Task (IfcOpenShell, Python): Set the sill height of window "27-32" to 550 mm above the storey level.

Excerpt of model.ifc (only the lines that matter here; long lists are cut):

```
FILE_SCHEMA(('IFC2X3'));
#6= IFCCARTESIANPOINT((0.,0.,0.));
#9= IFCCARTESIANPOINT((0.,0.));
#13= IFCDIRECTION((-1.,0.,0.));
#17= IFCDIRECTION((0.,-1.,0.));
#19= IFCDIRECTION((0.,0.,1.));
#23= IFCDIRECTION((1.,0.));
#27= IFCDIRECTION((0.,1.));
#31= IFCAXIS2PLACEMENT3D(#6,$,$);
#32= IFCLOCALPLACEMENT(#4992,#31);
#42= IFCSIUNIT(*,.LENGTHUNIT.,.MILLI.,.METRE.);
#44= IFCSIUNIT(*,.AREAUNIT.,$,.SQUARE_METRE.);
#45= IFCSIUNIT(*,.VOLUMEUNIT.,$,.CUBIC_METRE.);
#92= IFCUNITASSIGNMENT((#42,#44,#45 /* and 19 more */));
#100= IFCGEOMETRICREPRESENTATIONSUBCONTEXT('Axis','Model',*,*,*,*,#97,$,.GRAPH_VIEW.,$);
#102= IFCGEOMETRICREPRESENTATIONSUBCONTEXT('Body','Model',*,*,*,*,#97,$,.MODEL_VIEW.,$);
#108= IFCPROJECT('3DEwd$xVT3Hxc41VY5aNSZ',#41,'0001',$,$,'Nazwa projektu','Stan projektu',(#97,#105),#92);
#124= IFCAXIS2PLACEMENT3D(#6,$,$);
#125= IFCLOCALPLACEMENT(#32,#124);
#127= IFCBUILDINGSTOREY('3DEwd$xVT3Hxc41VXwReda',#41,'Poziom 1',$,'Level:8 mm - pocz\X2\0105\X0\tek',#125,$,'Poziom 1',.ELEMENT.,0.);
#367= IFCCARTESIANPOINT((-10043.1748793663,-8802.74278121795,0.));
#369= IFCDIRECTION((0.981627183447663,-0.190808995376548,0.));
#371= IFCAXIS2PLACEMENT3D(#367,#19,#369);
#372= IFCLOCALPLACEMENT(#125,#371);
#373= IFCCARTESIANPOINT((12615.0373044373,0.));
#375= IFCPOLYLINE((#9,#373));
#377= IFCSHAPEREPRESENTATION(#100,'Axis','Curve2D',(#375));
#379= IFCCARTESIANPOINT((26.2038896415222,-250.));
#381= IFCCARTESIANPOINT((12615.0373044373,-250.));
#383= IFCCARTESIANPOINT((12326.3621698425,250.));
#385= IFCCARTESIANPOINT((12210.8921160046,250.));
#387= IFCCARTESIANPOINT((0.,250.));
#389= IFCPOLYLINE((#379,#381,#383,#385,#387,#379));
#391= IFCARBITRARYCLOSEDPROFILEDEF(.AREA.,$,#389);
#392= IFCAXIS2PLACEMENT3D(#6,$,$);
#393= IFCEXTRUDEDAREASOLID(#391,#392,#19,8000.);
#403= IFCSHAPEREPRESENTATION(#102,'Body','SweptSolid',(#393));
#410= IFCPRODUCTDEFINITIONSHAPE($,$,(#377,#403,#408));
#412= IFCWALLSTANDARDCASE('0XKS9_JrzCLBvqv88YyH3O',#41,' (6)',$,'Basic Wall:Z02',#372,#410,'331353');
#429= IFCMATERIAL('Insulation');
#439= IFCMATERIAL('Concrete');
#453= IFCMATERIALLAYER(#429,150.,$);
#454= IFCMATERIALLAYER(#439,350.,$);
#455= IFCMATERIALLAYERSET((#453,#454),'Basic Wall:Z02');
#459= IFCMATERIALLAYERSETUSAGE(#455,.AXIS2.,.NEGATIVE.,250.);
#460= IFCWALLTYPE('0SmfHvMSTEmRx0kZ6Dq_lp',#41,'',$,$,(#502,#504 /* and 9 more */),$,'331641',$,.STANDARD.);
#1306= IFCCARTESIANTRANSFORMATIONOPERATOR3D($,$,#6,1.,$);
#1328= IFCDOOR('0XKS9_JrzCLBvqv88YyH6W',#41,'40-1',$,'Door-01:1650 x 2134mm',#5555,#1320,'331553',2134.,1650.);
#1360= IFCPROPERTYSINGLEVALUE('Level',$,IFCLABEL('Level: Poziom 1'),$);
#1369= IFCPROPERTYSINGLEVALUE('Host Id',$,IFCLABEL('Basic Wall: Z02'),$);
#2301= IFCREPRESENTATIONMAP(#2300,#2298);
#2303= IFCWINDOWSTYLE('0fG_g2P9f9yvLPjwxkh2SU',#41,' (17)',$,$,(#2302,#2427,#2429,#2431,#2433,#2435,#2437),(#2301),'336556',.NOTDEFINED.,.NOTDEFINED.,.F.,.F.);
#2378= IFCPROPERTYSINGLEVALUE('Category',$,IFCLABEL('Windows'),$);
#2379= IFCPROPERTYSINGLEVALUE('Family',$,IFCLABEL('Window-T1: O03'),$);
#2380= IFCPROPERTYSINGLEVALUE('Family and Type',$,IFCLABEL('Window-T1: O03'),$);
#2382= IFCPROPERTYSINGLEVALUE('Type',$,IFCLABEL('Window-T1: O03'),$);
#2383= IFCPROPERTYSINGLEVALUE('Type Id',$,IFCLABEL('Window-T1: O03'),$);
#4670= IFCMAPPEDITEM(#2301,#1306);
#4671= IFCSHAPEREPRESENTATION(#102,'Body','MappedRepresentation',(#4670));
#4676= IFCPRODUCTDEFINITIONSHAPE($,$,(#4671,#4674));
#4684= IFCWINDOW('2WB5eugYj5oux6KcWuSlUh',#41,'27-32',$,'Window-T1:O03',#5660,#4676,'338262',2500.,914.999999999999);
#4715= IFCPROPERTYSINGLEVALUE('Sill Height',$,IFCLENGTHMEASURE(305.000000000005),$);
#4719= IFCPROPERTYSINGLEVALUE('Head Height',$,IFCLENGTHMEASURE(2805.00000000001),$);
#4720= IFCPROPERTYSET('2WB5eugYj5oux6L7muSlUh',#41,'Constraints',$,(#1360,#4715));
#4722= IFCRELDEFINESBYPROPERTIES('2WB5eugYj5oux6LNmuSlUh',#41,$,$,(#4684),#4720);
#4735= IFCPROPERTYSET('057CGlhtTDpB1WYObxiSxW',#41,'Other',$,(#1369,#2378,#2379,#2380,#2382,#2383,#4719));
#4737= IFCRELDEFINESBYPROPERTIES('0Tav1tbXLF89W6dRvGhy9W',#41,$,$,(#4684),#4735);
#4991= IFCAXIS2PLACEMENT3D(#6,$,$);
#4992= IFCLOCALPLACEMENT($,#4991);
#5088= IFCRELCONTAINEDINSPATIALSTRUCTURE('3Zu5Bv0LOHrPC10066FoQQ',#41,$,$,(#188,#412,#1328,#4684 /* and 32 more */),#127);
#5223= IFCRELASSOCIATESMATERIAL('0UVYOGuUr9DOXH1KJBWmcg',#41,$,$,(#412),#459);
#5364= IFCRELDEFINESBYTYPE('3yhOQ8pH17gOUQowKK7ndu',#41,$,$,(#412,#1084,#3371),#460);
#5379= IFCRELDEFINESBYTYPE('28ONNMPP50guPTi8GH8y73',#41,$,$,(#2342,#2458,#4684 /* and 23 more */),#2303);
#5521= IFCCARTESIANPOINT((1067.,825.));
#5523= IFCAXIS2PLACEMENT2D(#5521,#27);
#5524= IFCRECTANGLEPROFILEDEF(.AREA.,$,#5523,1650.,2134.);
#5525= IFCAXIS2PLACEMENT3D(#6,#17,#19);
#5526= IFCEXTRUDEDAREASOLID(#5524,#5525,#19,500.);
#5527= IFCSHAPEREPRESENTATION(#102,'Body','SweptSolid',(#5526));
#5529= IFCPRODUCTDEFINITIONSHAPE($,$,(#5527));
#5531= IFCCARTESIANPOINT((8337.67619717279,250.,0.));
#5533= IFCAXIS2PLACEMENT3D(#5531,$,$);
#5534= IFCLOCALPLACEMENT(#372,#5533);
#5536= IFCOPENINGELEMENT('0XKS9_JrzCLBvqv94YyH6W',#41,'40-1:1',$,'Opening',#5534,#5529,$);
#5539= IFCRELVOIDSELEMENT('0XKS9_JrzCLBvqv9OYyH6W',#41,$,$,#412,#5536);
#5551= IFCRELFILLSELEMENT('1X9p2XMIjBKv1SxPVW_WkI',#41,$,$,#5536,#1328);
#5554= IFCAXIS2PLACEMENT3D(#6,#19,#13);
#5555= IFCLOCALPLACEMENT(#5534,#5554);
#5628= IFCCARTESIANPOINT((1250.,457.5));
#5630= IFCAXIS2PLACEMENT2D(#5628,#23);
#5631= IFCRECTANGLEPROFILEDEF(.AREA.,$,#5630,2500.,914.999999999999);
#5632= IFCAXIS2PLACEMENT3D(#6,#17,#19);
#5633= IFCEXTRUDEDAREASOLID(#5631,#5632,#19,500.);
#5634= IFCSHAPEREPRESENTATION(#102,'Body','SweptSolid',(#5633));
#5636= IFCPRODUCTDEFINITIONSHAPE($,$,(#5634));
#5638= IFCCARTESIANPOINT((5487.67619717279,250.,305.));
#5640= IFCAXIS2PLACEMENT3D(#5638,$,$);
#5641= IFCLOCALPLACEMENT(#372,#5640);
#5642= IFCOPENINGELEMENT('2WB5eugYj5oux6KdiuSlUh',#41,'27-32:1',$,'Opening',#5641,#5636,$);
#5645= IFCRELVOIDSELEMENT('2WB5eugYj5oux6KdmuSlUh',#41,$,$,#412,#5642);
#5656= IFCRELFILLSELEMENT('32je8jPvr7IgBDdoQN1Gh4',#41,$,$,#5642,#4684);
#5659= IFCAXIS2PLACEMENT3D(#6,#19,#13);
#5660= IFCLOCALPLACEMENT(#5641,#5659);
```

```python
import numpy as np
import ifcopenshell
import ifcopenshell.api.geometry
import ifcopenshell.api.pset
import ifcopenshell.geom
import ifcopenshell.util.element
import ifcopenshell.util.placement
import ifcopenshell.util.shape
import ifcopenshell.util.unit

model = ifcopenshell.open("model.ifc")
unit_scale = ifcopenshell.util.unit.calculate_unit_scale(model)

window = model.by_guid("2WB5eugYj5oux6KcWuSlUh")
opening = window.FillsVoids[0].RelatingOpeningElement
storey = ifcopenshell.util.element.get_container(window, ifc_class="IfcBuildingStorey")
level = ifcopenshell.util.placement.get_local_placement(storey.ObjectPlacement)[2, 3]

# The opening's origin need not be at the sill, so measure its lowest point.
shape = ifcopenshell.geom.create_shape(ifcopenshell.geom.settings(), opening)
bottom = ifcopenshell.util.shape.get_shape_bottom_elevation(shape, shape.geometry) / unit_scale
dz = level + 0.55 / unit_scale - bottom

shift = np.array([0.0, 0.0, dz])
# The window is placed relative to its opening, so it follows when the opening moves.
matrix = ifcopenshell.util.placement.get_local_placement(opening.ObjectPlacement)
matrix[:3, 3] += shift
ifcopenshell.api.geometry.edit_object_placement(
    model, product=opening, matrix=matrix, is_si=False, should_transform_children=True
)

# Keep the stored heights in step.
pset = model.by_id(ifcopenshell.util.element.get_pset(window, "Constraints", should_inherit=False)["id"])
ifcopenshell.api.pset.edit_pset(model, pset=pset, properties={
    "Sill Height": model.create_entity("IfcLengthMeasure", ifcopenshell.util.element.get_pset(window, "Constraints", "Sill Height") + dz),
})
pset = model.by_id(ifcopenshell.util.element.get_pset(window, "Other", should_inherit=False)["id"])
ifcopenshell.api.pset.edit_pset(model, pset=pset, properties={
    "Head Height": model.create_entity("IfcLengthMeasure", ifcopenshell.util.element.get_pset(window, "Other", "Head Height") + dz),
})

print(f"moved by {dz * unit_scale:+.3f} m")

model.write("model_edited.ifc")
```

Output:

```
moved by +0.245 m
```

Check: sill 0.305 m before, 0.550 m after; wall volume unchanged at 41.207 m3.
